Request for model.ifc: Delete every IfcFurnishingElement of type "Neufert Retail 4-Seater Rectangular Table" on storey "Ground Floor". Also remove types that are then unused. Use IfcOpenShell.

First a look at what the model holds.

```python
import ifcopenshell
import ifcopenshell.util.element

model = ifcopenshell.open("model.ifc")
print(model.schema)
storey = next(s for s in model.by_type("IfcBuildingStorey") if s.Name == "Ground Floor")
furniture = [e for e in ifcopenshell.util.element.get_decomposition(storey) if e.is_a("IfcFurnishingElement")]
seen = {}
for e in furniture:
    element_type = ifcopenshell.util.element.get_type(e)
    name = element_type.Name if element_type not in (None, e) else None
    seen[name] = seen.get(name, 0) + 1
for name, count in sorted(seen.items(), key=str):
    print(count, "x", name)
```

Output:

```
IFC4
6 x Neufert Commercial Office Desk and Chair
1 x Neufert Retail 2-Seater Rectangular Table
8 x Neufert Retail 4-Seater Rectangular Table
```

```python
import ifcopenshell
import ifcopenshell.api.root
import ifcopenshell.util.element

model = ifcopenshell.open("model.ifc")

storey = next(s for s in model.by_type("IfcBuildingStorey") if s.Name == "Ground Floor")
furniture = [e for e in ifcopenshell.util.element.get_decomposition(storey) if e.is_a("IfcFurnishingElement")]
targets = [e for e in furniture if (t := ifcopenshell.util.element.get_type(e)) not in (None, e) and t.Name == "Neufert Retail 4-Seater Rectangular Table"]
types = {ifcopenshell.util.element.get_type(e) for e in targets} - {None, *targets}

for e in targets:
    ifcopenshell.api.root.remove_product(model, product=e)
print(len(targets), "removed")

unused = [t for t in types if not ifcopenshell.util.element.get_types(t)]
for t in unused:
    ifcopenshell.api.root.remove_product(model, product=t)
print(len(unused), "unused types removed")

model.write("model-out.ifc")
```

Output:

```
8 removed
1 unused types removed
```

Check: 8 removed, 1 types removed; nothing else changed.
